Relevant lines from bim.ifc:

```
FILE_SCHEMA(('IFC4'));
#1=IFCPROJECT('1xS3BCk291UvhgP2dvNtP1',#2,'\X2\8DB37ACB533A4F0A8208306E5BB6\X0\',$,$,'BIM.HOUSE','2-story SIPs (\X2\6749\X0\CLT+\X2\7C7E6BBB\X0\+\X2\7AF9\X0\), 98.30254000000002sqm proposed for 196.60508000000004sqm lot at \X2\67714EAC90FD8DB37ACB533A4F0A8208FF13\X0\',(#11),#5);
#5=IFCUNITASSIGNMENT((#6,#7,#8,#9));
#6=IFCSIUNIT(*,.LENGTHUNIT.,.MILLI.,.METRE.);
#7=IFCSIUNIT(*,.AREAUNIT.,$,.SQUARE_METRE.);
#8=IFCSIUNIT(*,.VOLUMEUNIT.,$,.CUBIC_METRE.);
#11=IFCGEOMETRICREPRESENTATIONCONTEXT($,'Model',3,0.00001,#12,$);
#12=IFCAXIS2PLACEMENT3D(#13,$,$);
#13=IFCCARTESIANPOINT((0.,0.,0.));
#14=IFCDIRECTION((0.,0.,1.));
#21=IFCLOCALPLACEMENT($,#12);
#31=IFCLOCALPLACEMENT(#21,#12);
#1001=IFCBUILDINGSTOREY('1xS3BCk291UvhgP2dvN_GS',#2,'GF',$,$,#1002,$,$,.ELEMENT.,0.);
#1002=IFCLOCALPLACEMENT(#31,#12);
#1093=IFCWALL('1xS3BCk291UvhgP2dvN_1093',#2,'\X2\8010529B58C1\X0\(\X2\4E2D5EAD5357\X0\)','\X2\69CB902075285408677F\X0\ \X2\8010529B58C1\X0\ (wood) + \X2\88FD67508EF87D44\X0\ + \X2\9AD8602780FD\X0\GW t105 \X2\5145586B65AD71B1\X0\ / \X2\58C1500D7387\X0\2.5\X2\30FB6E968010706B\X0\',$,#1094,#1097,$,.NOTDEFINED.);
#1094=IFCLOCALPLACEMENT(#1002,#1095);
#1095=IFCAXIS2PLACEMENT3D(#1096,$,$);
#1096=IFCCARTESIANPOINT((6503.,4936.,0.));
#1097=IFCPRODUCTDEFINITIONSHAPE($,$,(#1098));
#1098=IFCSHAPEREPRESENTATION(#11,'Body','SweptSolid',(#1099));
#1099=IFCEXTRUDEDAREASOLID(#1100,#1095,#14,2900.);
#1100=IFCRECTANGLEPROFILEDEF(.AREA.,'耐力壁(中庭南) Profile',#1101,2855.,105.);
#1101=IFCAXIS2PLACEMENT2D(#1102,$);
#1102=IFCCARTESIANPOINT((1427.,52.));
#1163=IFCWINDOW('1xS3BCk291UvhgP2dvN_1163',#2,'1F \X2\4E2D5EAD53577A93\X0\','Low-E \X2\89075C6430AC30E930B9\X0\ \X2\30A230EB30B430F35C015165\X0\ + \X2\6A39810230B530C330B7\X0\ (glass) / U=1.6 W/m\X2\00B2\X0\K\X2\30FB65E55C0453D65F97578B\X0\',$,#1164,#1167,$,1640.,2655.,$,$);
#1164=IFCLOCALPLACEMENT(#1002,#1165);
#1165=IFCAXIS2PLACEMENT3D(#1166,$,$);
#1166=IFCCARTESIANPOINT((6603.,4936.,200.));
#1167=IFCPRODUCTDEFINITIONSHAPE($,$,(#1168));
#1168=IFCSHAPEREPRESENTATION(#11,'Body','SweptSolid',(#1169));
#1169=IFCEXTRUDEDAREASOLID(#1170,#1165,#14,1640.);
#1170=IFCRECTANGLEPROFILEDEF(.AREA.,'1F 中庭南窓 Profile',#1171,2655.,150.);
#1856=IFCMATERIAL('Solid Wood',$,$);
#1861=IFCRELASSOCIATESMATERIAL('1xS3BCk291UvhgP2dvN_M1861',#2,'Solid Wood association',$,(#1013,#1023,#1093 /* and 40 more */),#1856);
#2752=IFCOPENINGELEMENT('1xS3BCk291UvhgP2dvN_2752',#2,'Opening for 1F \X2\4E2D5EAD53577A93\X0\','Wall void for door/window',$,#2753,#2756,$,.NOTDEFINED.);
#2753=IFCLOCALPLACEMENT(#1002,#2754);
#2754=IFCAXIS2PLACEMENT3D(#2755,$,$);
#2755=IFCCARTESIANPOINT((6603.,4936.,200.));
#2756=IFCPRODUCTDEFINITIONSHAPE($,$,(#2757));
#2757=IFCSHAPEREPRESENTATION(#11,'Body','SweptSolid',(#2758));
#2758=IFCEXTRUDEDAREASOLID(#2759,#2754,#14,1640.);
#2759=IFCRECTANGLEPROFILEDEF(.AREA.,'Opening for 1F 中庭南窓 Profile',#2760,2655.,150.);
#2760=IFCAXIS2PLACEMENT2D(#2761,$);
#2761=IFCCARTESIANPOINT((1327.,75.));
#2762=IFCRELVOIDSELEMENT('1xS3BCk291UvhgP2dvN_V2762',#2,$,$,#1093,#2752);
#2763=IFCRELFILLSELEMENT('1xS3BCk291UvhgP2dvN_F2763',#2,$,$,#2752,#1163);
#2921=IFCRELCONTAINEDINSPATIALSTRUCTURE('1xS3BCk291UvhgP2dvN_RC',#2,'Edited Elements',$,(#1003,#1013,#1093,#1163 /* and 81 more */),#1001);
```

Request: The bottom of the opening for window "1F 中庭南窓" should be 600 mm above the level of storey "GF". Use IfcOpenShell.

```python
import numpy as np
import ifcopenshell
import ifcopenshell.api.geometry
import ifcopenshell.geom
import ifcopenshell.util.element
import ifcopenshell.util.placement
import ifcopenshell.util.shape
import ifcopenshell.util.unit

model = ifcopenshell.open("bim.ifc")
unit_scale = ifcopenshell.util.unit.calculate_unit_scale(model)

window = model.by_guid("1xS3BCk291UvhgP2dvN_1163")
opening = window.FillsVoids[0].RelatingOpeningElement
storey = ifcopenshell.util.element.get_container(window, ifc_class="IfcBuildingStorey")
level = ifcopenshell.util.placement.get_local_placement(storey.ObjectPlacement)[2, 3]

# The opening's origin need not be at the sill, so measure its lowest point.
shape = ifcopenshell.geom.create_shape(ifcopenshell.geom.settings(), opening)
bottom = ifcopenshell.util.shape.get_shape_bottom_elevation(shape, shape.geometry) / unit_scale
dz = level + 0.6 / unit_scale - bottom

shift = np.array([0.0, 0.0, dz])
# The window is not placed relative to its opening, so move both.
for product in (opening, window):
    matrix = ifcopenshell.util.placement.get_local_placement(product.ObjectPlacement)
    matrix[:3, 3] += shift
    ifcopenshell.api.geometry.edit_object_placement(model, product=product, matrix=matrix, is_si=False)

print(f"moved by {dz * unit_scale:+.3f} m")

model.write("bim_updated.ifc")
```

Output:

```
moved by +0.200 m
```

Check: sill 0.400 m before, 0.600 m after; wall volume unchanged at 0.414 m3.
